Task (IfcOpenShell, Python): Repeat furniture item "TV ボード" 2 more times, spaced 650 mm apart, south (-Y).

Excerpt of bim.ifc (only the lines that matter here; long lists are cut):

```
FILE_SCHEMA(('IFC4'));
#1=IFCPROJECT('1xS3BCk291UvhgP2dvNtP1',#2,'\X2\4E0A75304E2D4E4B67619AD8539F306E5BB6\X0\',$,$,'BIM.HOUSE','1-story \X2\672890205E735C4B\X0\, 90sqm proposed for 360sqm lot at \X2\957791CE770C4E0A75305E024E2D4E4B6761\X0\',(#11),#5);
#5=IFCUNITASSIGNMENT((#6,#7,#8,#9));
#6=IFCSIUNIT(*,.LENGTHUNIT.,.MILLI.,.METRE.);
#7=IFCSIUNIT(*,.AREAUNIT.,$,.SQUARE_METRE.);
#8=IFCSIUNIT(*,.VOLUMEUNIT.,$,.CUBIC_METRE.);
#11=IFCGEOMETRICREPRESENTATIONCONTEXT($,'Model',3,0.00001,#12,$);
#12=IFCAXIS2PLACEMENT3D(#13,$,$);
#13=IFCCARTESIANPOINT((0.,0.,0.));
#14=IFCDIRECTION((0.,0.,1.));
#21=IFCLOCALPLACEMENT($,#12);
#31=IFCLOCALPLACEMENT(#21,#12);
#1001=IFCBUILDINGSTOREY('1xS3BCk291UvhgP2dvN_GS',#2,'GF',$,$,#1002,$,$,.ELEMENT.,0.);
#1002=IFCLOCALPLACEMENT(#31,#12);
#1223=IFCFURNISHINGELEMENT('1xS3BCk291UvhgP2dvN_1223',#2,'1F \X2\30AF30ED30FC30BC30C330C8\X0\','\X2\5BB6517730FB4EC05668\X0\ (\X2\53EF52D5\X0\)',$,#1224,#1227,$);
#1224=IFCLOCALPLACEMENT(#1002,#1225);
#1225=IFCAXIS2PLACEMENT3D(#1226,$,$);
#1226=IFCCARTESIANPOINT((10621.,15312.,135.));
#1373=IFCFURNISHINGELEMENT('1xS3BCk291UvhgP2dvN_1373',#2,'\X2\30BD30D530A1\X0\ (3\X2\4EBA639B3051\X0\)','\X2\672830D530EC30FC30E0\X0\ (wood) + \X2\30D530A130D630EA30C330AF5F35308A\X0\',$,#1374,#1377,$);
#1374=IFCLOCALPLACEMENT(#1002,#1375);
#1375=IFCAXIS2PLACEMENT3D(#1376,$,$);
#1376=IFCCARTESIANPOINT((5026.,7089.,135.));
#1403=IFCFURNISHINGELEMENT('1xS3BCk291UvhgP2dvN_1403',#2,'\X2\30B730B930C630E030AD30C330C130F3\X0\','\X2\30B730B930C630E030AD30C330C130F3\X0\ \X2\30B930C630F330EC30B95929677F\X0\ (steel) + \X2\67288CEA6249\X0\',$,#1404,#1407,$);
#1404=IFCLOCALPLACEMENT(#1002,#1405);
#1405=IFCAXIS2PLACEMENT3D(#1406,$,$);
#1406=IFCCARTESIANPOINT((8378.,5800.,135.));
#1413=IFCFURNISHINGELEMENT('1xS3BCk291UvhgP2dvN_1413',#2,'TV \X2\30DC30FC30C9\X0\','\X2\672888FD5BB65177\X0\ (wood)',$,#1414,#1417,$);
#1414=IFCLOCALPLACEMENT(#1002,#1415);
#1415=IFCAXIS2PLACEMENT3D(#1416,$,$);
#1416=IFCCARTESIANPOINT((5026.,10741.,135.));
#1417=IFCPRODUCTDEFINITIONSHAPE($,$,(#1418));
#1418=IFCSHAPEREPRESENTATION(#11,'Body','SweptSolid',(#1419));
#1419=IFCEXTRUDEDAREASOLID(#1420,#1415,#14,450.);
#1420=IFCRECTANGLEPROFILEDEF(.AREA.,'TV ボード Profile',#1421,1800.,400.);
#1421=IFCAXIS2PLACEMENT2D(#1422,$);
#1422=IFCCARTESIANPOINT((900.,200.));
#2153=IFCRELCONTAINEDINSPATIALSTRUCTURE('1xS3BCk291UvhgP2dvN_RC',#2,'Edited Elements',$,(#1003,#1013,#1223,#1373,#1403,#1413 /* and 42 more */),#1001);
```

```python
import numpy as np
import ifcopenshell
import ifcopenshell.api.geometry
import ifcopenshell.api.root
import ifcopenshell.util.element
import ifcopenshell.util.placement
import ifcopenshell.util.unit

model = ifcopenshell.open("bim.ifc")
unit_scale = ifcopenshell.util.unit.calculate_unit_scale(model)


def reuse_history(source, copy):
    """copy_class also copies each property set's owner history, people and application; keep the originals."""
    for rel in copy.IsDefinedBy:
        if rel.is_a("IfcRelDefinesByProperties") and (history := rel.RelatingPropertyDefinition.OwnerHistory):
            rel.RelatingPropertyDefinition.OwnerHistory = source.OwnerHistory
            ifcopenshell.util.element.remove_deep2(model, history)


source = model.by_id(1413)
base = ifcopenshell.util.placement.get_local_placement(source.ObjectPlacement)
step = np.array([0.0, -1.0, 0.0]) * 0.65 / unit_scale

for i in range(1, 3):
    copy = ifcopenshell.api.root.copy_class(model, product=source)
    copy.Representation = ifcopenshell.util.element.copy_deep(
        model, source.Representation, exclude=["IfcGeometricRepresentationContext", "IfcRepresentationMap"]
    )
    reuse_history(source, copy)
    matrix = base.copy()
    matrix[:3, 3] += i * step
    print("added at", matrix[:3, 3].round(3) + 0.0)
    ifcopenshell.api.geometry.edit_object_placement(model, product=copy, matrix=matrix, is_si=False)

model.write("bim-out.ifc")
```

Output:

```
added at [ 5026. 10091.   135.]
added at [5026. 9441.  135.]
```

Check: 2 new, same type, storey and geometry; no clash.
